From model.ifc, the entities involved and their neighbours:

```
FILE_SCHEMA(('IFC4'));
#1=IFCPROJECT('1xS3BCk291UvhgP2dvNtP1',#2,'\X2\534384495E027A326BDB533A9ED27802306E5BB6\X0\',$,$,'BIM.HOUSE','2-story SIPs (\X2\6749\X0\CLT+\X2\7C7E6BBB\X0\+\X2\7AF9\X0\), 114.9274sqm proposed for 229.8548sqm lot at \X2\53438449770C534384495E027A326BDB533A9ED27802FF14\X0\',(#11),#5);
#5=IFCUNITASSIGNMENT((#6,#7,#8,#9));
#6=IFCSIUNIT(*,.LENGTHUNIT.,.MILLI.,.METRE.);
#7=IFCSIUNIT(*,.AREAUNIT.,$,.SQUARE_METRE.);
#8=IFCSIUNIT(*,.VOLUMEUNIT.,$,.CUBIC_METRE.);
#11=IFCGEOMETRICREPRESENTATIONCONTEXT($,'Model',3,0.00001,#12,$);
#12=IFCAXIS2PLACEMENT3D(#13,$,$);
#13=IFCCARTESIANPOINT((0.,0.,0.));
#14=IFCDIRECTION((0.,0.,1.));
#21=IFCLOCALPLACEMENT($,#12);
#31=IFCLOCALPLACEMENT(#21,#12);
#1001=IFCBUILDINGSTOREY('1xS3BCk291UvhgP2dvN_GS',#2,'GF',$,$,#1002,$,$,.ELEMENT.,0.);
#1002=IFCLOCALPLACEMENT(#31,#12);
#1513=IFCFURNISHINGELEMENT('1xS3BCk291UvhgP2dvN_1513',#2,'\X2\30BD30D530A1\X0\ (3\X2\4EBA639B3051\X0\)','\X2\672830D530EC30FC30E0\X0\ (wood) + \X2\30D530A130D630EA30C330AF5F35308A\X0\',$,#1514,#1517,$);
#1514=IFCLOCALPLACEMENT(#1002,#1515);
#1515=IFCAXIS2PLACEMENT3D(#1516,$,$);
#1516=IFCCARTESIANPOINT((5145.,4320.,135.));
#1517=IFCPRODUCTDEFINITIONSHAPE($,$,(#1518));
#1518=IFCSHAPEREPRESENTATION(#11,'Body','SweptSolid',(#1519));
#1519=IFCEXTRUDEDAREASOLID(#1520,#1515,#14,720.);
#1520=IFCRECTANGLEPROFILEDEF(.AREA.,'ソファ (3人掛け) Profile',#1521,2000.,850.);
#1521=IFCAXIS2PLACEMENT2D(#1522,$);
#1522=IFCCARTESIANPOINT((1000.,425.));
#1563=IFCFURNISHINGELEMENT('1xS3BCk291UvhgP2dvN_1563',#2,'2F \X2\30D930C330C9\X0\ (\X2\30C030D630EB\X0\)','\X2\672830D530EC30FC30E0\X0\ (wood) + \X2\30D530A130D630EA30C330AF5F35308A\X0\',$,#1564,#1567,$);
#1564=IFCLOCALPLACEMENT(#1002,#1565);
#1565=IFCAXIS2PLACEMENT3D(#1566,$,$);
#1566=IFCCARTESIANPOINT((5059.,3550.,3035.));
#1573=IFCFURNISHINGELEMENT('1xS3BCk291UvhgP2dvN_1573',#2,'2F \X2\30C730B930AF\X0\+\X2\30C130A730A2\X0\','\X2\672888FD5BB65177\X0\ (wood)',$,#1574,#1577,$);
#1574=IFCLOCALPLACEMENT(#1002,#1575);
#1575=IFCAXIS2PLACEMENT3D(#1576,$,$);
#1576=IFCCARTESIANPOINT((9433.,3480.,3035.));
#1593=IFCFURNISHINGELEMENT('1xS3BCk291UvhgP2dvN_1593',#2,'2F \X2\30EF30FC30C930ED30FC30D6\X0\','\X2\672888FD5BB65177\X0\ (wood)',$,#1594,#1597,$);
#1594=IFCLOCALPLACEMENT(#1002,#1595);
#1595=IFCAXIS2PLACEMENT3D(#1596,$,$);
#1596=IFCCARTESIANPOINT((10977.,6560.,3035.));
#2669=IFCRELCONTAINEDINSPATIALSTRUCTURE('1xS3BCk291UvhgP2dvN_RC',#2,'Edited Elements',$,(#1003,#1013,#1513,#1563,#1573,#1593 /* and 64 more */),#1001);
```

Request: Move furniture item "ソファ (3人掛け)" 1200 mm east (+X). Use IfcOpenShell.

```python
import ifcopenshell
import ifcopenshell.api.geometry
import ifcopenshell.util.placement
import ifcopenshell.util.unit

model = ifcopenshell.open("model.ifc")
unit_scale = ifcopenshell.util.unit.calculate_unit_scale(model)

item = model.by_guid("1xS3BCk291UvhgP2dvN_1513")
matrix = ifcopenshell.util.placement.get_local_placement(item.ObjectPlacement)
matrix[0, 3] += 1.2 / unit_scale
ifcopenshell.api.geometry.edit_object_placement(model, product=item, matrix=matrix, is_si=False)

print(ifcopenshell.util.placement.get_local_placement(item.ObjectPlacement).round(3) + 0.0)

model.write("model-out.ifc")
```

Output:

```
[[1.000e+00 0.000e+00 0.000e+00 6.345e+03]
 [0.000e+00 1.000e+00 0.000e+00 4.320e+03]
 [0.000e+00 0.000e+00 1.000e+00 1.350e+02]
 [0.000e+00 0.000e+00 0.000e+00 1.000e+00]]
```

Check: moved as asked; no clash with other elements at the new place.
